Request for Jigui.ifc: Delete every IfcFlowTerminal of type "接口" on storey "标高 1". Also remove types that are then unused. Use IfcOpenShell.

First a look at what the model holds.

```python
import ifcopenshell
import ifcopenshell.util.element

model = ifcopenshell.open("Jigui.ifc")
print(model.schema)
storey = next(s for s in model.by_type("IfcBuildingStorey") if s.Name == "标高 1")
terminals = [e for e in ifcopenshell.util.element.get_decomposition(storey) if e.is_a("IfcFlowTerminal")]
seen = {}
for e in terminals:
    element_type = ifcopenshell.util.element.get_type(e)
    name = element_type.Name if element_type not in (None, e) else None
    seen[name] = seen.get(name, 0) + 1
for name, count in sorted(seen.items(), key=str):
    print(count, "x", name)
```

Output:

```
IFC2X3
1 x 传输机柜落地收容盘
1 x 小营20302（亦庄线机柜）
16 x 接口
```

```python
import ifcopenshell
import ifcopenshell.api.root
import ifcopenshell.util.element

model = ifcopenshell.open("Jigui.ifc")

storey = next(s for s in model.by_type("IfcBuildingStorey") if s.Name == "标高 1")
terminals = [e for e in ifcopenshell.util.element.get_decomposition(storey) if e.is_a("IfcFlowTerminal")]
targets = [e for e in terminals if (t := ifcopenshell.util.element.get_type(e)) not in (None, e) and t.Name == "接口"]
types = {ifcopenshell.util.element.get_type(e) for e in targets} - {None, *targets}

for e in targets:
    ifcopenshell.api.root.remove_product(model, product=e)
print(len(targets), "removed")

unused = [t for t in types if not ifcopenshell.util.element.get_types(t)]
for t in unused:
    ifcopenshell.api.root.remove_product(model, product=t)
print(len(unused), "unused types removed")

model.write("Jigui_v2.ifc")
```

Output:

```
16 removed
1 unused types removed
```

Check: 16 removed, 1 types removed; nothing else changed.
